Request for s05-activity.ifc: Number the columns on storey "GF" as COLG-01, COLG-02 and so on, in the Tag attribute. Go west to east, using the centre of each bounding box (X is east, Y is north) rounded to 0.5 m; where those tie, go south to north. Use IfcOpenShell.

First a look at what the model holds.

```python
import ifcopenshell
import ifcopenshell.util.element
import ifcopenshell.util.placement

model = ifcopenshell.open("s05-activity.ifc")
print(model.schema)
storey = next(s for s in model.by_type("IfcBuildingStorey") if s.Name == "GF")
columns = [e for e in ifcopenshell.util.element.get_decomposition(storey) if e.is_a("IfcColumn")]
for e in sorted(columns, key=lambda e: e.id()):
    origin = ifcopenshell.util.placement.get_local_placement(e.ObjectPlacement)[:3, 3]
    print(e.id(), e.Tag, e.Name, origin.round(2) + 0.0, sep=" | ")
```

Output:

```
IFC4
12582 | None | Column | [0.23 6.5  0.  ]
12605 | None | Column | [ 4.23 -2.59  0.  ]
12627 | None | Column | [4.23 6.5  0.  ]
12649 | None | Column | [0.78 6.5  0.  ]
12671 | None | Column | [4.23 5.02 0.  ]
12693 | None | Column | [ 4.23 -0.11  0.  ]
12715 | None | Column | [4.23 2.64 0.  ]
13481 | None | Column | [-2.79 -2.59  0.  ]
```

```python
import ifcopenshell
import ifcopenshell.geom
import ifcopenshell.util.element
import ifcopenshell.util.shape

model = ifcopenshell.open("s05-activity.ifc")
settings = ifcopenshell.geom.settings()
settings.set("use-world-coords", True)


def centre(element):
    shape = ifcopenshell.geom.create_shape(settings, element)
    return ifcopenshell.util.shape.get_bbox_centroid(shape.geometry)


storey = next(s for s in model.by_type("IfcBuildingStorey") if s.Name == "GF")
columns = [e for e in ifcopenshell.util.element.get_decomposition(storey) if e.is_a("IfcColumn")]

# Insertion points can sit at a corner or the storey origin, so sort by the geometry (in metres).
centres = {e: centre(e) for e in columns}
columns.sort(key=lambda e: (round(centres[e][0] / 0.5), centres[e][1]))

for i, e in enumerate(columns, start=1):
    number = f"COLG-{i:02d}"
    e.Tag = number
    print(e.id(), number)

model.write("s05-activity-out.ifc")
```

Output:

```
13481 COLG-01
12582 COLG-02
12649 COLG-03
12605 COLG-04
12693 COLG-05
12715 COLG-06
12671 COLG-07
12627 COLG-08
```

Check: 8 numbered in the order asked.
